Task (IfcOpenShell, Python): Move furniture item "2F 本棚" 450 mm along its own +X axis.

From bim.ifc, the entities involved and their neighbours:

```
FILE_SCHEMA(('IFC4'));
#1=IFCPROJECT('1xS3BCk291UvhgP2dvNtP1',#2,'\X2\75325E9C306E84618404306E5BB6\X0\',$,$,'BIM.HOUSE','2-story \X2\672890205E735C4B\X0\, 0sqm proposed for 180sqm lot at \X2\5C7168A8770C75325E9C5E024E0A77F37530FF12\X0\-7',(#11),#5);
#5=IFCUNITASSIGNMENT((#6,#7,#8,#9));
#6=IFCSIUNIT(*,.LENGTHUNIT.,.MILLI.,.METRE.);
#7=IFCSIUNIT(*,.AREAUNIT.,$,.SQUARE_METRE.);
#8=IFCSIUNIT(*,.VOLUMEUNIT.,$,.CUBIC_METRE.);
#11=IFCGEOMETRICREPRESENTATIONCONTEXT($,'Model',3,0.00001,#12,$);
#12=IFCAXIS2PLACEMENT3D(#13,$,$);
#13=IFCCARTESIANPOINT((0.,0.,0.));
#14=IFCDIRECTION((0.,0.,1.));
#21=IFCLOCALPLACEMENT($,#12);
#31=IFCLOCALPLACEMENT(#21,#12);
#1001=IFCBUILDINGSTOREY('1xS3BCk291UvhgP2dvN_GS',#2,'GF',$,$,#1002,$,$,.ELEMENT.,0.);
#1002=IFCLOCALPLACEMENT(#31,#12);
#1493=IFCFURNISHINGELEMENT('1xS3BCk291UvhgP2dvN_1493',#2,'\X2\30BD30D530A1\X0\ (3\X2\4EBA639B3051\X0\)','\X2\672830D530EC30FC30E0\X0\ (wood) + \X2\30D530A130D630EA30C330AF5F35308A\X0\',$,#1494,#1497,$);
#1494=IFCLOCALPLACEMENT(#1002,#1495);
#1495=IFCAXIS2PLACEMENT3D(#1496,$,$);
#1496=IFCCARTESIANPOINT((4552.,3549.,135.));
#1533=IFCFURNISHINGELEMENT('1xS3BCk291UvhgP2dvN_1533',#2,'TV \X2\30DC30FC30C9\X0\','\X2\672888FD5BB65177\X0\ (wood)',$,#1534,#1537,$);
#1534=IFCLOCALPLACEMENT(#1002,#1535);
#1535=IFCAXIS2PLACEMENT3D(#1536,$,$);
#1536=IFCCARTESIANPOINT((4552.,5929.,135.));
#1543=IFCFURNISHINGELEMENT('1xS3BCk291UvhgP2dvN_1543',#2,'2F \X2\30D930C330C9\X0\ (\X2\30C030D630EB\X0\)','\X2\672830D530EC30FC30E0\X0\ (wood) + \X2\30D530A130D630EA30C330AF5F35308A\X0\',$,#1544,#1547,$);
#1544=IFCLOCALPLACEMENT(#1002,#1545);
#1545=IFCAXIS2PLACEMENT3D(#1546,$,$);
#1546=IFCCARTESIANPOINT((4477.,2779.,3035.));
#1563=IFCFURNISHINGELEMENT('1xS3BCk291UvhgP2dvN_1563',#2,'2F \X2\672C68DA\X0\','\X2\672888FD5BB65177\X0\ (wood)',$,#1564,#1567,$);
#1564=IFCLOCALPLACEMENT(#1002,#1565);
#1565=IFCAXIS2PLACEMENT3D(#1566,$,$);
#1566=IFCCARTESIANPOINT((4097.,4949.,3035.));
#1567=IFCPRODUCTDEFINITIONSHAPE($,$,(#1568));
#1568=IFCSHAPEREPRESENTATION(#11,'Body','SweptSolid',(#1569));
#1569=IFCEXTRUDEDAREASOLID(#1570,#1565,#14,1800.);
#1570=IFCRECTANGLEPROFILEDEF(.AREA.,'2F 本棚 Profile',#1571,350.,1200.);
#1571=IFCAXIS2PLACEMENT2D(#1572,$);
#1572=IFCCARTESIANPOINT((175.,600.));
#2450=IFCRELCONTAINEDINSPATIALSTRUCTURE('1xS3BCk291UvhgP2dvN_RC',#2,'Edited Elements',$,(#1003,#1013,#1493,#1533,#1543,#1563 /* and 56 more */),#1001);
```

```python
import ifcopenshell
import ifcopenshell.api.geometry
import ifcopenshell.util.placement
import ifcopenshell.util.unit

model = ifcopenshell.open("bim.ifc")
unit_scale = ifcopenshell.util.unit.calculate_unit_scale(model)

item = model.by_guid("1xS3BCk291UvhgP2dvN_1563")
matrix = ifcopenshell.util.placement.get_local_placement(item.ObjectPlacement)
matrix[:3, 3] += matrix[:3, 0] * 0.45 / unit_scale
ifcopenshell.api.geometry.edit_object_placement(model, product=item, matrix=matrix, is_si=False)

print(ifcopenshell.util.placement.get_local_placement(item.ObjectPlacement).round(3) + 0.0)

model.write("bim_v2.ifc")
```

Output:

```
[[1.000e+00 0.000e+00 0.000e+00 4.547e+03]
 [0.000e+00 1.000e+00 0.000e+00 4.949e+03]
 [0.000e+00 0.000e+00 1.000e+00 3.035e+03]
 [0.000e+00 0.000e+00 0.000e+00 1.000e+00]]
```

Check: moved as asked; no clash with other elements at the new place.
